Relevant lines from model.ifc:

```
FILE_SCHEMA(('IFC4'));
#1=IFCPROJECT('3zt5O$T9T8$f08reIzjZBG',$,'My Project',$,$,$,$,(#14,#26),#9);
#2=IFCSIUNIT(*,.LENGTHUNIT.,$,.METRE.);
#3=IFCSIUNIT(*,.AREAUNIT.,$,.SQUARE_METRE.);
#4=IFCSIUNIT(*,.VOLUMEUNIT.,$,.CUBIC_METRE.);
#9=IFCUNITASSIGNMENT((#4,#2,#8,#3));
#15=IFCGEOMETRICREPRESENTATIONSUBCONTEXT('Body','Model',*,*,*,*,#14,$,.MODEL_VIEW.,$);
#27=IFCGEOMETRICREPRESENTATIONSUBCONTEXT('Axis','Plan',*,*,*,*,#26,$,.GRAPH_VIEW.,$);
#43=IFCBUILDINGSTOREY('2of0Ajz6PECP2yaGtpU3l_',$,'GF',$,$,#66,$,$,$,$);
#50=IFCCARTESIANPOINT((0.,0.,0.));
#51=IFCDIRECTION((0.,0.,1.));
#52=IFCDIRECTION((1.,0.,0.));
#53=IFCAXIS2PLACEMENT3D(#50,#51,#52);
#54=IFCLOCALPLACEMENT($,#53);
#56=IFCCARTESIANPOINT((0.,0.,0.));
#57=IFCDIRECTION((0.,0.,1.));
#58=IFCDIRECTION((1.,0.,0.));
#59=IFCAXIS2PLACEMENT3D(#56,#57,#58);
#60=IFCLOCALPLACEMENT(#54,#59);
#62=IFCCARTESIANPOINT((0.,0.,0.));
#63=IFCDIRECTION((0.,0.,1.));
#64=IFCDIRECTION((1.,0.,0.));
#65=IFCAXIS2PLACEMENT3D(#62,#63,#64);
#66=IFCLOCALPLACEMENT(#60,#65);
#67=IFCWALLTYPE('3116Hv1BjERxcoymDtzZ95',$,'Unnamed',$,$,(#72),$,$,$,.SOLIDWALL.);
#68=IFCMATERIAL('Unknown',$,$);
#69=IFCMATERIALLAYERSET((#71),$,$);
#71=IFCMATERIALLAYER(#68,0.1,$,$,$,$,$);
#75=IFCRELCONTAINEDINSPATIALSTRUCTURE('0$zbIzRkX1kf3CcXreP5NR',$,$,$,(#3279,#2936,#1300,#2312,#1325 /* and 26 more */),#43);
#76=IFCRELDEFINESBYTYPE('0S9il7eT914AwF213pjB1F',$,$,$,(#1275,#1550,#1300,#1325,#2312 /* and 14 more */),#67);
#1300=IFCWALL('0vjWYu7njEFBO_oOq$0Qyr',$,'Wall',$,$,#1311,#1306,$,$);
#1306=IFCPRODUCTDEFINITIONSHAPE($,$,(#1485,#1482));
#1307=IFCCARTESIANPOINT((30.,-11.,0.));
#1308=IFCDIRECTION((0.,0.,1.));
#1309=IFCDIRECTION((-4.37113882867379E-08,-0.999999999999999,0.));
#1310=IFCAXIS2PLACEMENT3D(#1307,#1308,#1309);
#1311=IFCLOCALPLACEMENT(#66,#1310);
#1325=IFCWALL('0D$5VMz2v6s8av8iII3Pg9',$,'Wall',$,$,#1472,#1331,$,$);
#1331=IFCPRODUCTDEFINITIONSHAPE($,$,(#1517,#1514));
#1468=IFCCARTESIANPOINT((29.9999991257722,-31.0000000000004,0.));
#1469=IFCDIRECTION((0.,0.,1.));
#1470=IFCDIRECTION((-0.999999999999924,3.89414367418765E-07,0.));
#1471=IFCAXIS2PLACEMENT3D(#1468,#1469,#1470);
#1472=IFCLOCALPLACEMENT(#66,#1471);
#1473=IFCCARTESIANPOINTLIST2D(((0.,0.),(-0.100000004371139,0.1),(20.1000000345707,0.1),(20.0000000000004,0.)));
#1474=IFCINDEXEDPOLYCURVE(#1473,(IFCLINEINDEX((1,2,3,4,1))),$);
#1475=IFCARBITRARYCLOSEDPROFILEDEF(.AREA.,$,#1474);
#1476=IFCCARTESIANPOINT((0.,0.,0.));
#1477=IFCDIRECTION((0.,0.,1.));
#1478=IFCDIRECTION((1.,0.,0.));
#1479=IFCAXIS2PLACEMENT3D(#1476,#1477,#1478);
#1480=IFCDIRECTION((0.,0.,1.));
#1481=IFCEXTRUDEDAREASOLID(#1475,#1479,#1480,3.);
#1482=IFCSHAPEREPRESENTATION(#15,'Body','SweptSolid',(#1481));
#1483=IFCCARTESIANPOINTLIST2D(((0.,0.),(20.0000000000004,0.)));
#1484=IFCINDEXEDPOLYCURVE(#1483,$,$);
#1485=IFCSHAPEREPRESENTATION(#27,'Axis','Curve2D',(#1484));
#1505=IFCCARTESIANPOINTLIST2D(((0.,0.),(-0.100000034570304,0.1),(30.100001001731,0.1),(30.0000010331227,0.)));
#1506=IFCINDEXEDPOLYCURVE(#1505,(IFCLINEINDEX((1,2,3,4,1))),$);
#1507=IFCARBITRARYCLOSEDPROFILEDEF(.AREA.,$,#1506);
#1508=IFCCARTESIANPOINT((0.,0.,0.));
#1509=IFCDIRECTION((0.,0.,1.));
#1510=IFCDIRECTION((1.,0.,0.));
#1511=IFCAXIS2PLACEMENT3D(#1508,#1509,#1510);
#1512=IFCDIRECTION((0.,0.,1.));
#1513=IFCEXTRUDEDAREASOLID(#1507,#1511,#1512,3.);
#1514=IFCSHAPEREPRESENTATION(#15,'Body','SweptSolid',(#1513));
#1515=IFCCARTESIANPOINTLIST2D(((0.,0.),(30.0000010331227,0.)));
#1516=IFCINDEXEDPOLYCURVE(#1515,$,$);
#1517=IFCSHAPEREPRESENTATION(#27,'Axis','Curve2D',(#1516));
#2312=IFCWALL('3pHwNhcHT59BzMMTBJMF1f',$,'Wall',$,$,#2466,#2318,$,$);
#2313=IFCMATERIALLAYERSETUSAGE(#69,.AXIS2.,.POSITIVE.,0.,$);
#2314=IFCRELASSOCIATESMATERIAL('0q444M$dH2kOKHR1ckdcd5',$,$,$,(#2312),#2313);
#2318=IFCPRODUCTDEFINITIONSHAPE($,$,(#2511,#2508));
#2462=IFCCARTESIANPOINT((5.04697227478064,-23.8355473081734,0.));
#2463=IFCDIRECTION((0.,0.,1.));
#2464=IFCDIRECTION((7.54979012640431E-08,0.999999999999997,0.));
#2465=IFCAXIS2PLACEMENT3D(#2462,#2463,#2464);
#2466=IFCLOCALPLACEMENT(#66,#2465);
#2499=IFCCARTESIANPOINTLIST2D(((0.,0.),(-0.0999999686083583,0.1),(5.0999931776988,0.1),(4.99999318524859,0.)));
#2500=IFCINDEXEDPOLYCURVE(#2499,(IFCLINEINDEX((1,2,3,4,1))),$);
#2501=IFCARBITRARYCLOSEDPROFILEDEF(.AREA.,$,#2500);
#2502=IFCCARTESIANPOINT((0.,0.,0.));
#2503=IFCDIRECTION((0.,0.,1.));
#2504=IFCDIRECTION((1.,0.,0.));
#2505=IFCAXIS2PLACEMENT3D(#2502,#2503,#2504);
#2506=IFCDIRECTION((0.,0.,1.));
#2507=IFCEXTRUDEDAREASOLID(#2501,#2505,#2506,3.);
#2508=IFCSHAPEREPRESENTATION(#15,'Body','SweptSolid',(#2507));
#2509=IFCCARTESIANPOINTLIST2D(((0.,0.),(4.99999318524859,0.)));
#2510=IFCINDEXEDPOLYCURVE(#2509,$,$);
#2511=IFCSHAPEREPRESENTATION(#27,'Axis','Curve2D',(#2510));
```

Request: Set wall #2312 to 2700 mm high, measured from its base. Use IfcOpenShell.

```python
import ifcopenshell
import ifcopenshell.geom
import ifcopenshell.util.representation
import ifcopenshell.util.shape
import ifcopenshell.util.unit

model = ifcopenshell.open("model.ifc")
unit_scale = ifcopenshell.util.unit.calculate_unit_scale(model)
settings = ifcopenshell.geom.settings()


def volume(element):
    """Net volume in cubic metres, openings subtracted."""
    shape = ifcopenshell.geom.create_shape(settings, element)
    return ifcopenshell.util.shape.get_volume(shape.geometry)


wall = model.by_guid("3pHwNhcHT59BzMMTBJMF1f")
before = volume(wall)

body = ifcopenshell.util.representation.get_representation(wall, "Model", "Body")
solid = body.Items[0]
old_height = solid.Depth
solid.Depth = 2.7 / unit_scale
after = volume(wall)

print(f"height {old_height:g} -> {solid.Depth:g}, volume {before:.3f} -> {after:.3f} m3")

model.write("model_updated.ifc")
```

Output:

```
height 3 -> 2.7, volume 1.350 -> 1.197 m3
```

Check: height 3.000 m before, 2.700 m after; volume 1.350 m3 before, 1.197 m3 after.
